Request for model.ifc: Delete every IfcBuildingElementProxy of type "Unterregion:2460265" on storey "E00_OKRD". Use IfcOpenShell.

First a look at what the model holds.

```python
import ifcopenshell
import ifcopenshell.util.element

model = ifcopenshell.open("model.ifc")
print(model.schema)
storey = next(s for s in model.by_type("IfcBuildingStorey") if s.Name == "E00_OKRD")
proxies = [e for e in ifcopenshell.util.element.get_decomposition(storey) if e.is_a("IfcBuildingElementProxy")]
seen = {}
for e in proxies:
    element_type = ifcopenshell.util.element.get_type(e)
    name = element_type.Name if element_type not in (None, e) else None
    seen[name] = seen.get(name, 0) + 1
for name, count in sorted(seen.items(), key=str):
    print(count, "x", name)
```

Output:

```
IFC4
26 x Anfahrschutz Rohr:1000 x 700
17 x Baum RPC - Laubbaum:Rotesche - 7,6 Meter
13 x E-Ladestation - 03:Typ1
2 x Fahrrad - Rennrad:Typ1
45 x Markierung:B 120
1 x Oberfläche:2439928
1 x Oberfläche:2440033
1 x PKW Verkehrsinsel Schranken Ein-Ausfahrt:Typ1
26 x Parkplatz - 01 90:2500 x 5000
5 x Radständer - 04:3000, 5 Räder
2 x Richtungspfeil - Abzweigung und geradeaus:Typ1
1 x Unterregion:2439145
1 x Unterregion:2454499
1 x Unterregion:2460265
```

```python
import ifcopenshell
import ifcopenshell.api.root
import ifcopenshell.util.element

model = ifcopenshell.open("model.ifc")

storey = next(s for s in model.by_type("IfcBuildingStorey") if s.Name == "E00_OKRD")
proxies = [e for e in ifcopenshell.util.element.get_decomposition(storey) if e.is_a("IfcBuildingElementProxy")]
targets = [e for e in proxies if (t := ifcopenshell.util.element.get_type(e)) not in (None, e) and t.Name == "Unterregion:2460265"]

for e in targets:
    ifcopenshell.api.root.remove_product(model, product=e)
print(len(targets), "removed")

model.write("model-out.ifc")
```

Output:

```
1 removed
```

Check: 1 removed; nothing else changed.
